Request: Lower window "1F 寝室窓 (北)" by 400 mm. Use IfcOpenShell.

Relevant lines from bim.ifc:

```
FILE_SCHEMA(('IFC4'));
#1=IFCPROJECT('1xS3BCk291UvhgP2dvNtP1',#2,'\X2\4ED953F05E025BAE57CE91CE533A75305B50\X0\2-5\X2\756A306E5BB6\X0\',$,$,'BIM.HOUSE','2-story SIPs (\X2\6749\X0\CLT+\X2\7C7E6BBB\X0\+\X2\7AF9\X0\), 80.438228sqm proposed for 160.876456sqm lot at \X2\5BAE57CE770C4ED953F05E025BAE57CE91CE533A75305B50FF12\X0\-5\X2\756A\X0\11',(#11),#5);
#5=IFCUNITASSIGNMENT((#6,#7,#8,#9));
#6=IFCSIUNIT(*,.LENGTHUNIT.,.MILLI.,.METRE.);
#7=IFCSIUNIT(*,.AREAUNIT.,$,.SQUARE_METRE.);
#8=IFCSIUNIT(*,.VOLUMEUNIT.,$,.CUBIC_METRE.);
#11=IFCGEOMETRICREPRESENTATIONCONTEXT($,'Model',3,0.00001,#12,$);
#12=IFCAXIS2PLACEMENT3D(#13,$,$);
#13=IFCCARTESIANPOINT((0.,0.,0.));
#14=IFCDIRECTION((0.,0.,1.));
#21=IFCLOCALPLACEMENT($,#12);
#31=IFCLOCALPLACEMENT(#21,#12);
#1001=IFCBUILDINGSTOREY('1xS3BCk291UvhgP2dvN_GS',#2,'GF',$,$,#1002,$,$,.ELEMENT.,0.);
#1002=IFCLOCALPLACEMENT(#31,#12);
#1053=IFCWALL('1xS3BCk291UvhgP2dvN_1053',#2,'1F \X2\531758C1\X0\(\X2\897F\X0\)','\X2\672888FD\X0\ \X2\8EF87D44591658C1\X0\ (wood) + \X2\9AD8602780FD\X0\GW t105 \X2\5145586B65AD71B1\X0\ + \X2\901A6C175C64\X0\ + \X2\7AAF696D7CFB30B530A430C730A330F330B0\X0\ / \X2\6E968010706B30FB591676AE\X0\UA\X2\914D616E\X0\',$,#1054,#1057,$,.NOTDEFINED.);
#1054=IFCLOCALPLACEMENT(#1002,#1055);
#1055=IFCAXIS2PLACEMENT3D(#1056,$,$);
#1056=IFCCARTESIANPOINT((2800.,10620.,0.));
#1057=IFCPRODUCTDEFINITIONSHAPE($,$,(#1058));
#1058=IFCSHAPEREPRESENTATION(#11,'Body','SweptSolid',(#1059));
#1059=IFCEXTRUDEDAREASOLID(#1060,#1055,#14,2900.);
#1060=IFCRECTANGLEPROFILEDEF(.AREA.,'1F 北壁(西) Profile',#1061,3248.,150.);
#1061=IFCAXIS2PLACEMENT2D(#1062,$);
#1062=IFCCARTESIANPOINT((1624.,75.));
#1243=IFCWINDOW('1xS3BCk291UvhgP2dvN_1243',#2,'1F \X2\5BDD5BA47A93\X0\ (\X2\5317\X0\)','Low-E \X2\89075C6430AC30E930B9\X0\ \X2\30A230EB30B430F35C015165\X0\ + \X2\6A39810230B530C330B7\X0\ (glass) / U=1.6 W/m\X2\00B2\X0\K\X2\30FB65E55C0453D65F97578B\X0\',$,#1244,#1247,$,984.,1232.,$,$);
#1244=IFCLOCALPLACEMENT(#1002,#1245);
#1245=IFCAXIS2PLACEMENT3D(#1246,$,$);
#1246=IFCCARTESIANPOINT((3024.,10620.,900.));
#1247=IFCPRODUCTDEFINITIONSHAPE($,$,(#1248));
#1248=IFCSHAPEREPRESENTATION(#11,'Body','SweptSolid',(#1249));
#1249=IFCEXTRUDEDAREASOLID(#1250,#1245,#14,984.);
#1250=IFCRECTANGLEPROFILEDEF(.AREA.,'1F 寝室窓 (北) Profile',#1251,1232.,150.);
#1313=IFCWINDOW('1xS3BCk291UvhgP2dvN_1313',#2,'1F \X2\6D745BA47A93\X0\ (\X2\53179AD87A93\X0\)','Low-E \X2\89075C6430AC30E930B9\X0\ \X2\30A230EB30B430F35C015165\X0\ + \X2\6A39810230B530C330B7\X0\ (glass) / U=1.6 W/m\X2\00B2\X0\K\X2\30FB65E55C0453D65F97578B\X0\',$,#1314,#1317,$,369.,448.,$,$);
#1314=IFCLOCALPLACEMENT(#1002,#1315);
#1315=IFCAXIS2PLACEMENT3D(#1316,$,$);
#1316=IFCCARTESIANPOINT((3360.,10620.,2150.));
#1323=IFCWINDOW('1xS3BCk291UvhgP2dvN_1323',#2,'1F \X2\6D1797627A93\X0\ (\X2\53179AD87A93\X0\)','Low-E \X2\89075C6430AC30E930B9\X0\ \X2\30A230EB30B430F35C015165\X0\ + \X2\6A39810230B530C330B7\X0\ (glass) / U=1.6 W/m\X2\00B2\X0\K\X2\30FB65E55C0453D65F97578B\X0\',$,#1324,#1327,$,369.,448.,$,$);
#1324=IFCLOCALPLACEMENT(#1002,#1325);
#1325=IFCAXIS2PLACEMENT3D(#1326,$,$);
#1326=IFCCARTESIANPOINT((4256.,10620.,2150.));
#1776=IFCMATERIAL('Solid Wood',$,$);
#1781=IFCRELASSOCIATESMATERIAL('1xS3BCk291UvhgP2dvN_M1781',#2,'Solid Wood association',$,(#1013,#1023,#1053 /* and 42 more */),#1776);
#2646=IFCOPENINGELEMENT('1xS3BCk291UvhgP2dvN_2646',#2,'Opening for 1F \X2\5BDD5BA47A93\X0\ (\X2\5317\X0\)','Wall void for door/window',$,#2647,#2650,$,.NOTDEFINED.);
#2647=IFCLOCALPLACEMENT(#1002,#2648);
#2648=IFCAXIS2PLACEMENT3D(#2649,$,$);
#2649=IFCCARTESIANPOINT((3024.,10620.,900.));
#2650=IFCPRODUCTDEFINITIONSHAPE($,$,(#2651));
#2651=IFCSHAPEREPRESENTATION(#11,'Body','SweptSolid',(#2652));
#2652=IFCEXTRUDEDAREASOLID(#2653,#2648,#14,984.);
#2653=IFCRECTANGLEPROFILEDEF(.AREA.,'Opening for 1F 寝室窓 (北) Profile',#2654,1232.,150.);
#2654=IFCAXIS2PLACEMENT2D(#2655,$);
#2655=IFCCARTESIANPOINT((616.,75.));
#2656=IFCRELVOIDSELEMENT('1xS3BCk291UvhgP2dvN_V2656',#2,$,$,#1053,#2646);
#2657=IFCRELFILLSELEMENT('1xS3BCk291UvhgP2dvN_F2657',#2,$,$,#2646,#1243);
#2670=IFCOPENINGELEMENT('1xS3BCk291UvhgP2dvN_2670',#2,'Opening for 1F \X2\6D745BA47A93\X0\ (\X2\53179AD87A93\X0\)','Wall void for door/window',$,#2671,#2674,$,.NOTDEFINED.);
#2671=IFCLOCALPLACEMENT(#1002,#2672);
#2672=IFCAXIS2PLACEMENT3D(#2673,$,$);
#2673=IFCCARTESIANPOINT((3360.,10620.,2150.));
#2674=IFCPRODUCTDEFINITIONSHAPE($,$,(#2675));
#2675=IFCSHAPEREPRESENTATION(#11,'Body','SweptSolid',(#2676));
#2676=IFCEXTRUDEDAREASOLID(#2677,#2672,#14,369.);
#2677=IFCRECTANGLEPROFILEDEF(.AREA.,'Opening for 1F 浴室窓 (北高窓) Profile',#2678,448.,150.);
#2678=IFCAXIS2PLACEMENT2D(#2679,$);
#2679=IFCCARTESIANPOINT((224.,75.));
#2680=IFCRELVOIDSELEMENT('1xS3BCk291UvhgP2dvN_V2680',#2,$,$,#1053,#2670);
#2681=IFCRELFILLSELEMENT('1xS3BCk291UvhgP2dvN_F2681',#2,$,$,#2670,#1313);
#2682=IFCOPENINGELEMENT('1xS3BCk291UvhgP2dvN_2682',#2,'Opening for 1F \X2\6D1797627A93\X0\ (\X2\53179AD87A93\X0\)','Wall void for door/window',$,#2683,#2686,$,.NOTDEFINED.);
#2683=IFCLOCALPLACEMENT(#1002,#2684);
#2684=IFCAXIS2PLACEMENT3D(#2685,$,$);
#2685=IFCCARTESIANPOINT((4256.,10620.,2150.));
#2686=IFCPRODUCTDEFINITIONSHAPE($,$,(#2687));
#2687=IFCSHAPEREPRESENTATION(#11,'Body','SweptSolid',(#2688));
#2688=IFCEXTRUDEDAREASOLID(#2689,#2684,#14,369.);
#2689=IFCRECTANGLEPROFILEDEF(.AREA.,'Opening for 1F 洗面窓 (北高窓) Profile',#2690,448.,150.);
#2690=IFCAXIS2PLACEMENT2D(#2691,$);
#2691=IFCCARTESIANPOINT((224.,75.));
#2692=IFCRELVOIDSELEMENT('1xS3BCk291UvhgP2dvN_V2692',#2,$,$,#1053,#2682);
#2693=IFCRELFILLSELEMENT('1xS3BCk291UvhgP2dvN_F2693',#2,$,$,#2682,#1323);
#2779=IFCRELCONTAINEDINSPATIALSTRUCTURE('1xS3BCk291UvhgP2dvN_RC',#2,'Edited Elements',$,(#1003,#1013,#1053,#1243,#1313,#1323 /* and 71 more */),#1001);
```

```python
import numpy as np
import ifcopenshell
import ifcopenshell.api.geometry
import ifcopenshell.util.placement
import ifcopenshell.util.unit

model = ifcopenshell.open("bim.ifc")
unit_scale = ifcopenshell.util.unit.calculate_unit_scale(model)

window = model.by_guid("1xS3BCk291UvhgP2dvN_1243")
opening = window.FillsVoids[0].RelatingOpeningElement
dz = -0.4 / unit_scale

shift = np.array([0.0, 0.0, dz])
# The window is not placed relative to its opening, so move both.
for product in (opening, window):
    matrix = ifcopenshell.util.placement.get_local_placement(product.ObjectPlacement)
    matrix[:3, 3] += shift
    ifcopenshell.api.geometry.edit_object_placement(model, product=product, matrix=matrix, is_si=False)

print(f"moved by {dz * unit_scale:+.3f} m")

model.write("bim_v2.ifc")
```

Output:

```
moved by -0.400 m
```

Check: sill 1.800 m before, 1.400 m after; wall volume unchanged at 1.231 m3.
